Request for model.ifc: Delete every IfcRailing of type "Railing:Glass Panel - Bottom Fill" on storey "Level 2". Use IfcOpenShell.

First a look at what the model holds.

```python
import ifcopenshell
import ifcopenshell.util.element

model = ifcopenshell.open("model.ifc")
print(model.schema)
storey = next(s for s in model.by_type("IfcBuildingStorey") if s.Name == "Level 2")
railings = [e for e in ifcopenshell.util.element.get_decomposition(storey) if e.is_a("IfcRailing")]
seen = {}
for e in railings:
    element_type = ifcopenshell.util.element.get_type(e)
    name = element_type.Name if element_type not in (None, e) else None
    seen[name] = seen.get(name, 0) + 1
for name, count in sorted(seen.items(), key=str):
    print(count, "x", name)
```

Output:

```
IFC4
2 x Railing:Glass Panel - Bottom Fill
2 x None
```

```python
import ifcopenshell
import ifcopenshell.api.root
import ifcopenshell.util.element

model = ifcopenshell.open("model.ifc")

storey = next(s for s in model.by_type("IfcBuildingStorey") if s.Name == "Level 2")
railings = [e for e in ifcopenshell.util.element.get_decomposition(storey) if e.is_a("IfcRailing")]
targets = [e for e in railings if (t := ifcopenshell.util.element.get_type(e)) not in (None, e) and t.Name == "Railing:Glass Panel - Bottom Fill"]

for e in targets:
    ifcopenshell.api.root.remove_product(model, product=e)
print(len(targets), "removed")

model.write("model_edited.ifc")
```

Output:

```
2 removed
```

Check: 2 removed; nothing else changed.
